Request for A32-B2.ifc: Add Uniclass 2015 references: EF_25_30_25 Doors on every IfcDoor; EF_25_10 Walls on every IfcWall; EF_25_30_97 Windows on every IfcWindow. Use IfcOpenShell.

First a look at what the model holds.

```python
import ifcopenshell

model = ifcopenshell.open("A32-B2.ifc")
print(model.schema)
print("classifications:", [c.Name for c in model.by_type("IfcClassification")])
for ifc_class in ("IfcDoor", "IfcRoof", "IfcStair", "IfcWall", "IfcWindow"):
    print(ifc_class, len(model.by_type(ifc_class)))
```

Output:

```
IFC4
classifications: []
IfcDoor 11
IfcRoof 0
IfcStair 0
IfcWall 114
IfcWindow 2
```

```python
import ifcopenshell
import ifcopenshell.api.classification

model = ifcopenshell.open("A32-B2.ifc")

system = ifcopenshell.api.classification.add_classification(model, classification="Uniclass 2015")

codes = {
    "IfcDoor": ("EF_25_30_25", "Doors"),
    "IfcWall": ("EF_25_10", "Walls"),
    "IfcWindow": ("EF_25_30_97", "Windows"),
}
for ifc_class, (code, name) in codes.items():
    products = model.by_type(ifc_class)
    ifcopenshell.api.classification.add_reference(
        model, products=products, classification=system, identification=code, name=name
    )
    print(code, len(products))

model.write("A32-B2_updated.ifc")
```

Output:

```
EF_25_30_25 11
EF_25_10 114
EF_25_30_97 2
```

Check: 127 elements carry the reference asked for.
